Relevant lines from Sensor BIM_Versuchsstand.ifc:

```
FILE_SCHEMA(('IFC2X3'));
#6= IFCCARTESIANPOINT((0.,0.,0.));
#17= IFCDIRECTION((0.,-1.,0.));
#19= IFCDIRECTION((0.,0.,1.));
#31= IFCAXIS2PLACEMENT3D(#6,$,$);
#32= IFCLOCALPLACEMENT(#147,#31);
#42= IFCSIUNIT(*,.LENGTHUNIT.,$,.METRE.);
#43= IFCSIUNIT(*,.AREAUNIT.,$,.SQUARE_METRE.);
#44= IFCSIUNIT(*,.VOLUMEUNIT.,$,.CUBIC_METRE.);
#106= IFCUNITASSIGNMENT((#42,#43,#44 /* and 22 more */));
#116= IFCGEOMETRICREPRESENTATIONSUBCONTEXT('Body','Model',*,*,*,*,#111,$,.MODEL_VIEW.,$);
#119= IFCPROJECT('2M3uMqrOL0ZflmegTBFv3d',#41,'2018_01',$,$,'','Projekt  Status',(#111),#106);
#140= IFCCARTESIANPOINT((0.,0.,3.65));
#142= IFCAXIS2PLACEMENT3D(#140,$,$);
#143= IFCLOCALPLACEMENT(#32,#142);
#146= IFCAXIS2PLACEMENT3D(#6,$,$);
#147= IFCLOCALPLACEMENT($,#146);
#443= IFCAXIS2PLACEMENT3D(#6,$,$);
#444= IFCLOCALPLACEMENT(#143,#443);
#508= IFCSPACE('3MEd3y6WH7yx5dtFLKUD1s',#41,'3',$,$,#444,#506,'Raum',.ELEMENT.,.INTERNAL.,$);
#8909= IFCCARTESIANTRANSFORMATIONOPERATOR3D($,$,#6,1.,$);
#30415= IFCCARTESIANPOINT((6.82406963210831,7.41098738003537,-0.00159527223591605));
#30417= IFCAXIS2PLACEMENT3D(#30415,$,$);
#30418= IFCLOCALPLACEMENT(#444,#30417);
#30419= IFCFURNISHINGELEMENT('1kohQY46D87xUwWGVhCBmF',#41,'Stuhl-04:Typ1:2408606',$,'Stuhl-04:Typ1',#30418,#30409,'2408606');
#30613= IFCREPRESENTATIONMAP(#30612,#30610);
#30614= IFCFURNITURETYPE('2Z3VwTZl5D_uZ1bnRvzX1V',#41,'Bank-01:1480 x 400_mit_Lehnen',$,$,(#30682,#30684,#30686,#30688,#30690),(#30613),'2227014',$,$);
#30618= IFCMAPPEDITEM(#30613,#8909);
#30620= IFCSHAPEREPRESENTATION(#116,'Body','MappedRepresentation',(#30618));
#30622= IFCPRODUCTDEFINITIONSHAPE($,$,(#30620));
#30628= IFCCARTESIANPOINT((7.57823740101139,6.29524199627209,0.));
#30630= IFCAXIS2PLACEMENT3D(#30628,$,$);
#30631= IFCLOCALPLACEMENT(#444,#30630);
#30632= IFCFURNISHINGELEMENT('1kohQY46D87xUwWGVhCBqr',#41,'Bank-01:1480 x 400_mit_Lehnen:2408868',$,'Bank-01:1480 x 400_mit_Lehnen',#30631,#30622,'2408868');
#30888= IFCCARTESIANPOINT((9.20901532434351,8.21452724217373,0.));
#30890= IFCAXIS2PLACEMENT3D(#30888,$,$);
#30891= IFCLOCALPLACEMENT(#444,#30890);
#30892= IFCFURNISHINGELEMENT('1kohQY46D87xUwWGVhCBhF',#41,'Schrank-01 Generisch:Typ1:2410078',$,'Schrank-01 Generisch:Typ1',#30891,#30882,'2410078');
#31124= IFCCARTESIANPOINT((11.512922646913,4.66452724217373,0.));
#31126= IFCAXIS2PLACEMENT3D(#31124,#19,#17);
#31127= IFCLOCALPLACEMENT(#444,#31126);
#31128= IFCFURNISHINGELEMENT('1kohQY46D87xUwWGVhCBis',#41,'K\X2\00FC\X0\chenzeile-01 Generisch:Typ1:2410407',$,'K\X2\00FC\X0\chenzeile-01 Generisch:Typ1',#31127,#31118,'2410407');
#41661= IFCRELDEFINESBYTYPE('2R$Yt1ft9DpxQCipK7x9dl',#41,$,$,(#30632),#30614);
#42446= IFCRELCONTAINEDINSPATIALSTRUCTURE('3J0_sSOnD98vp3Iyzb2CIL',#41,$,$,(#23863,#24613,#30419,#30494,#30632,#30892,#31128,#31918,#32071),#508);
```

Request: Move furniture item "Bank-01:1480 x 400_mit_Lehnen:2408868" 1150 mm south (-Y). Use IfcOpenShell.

```python
import ifcopenshell
import ifcopenshell.api.geometry
import ifcopenshell.util.placement
import ifcopenshell.util.unit

model = ifcopenshell.open("Sensor BIM_Versuchsstand.ifc")
unit_scale = ifcopenshell.util.unit.calculate_unit_scale(model)

item = model.by_guid("1kohQY46D87xUwWGVhCBqr")
matrix = ifcopenshell.util.placement.get_local_placement(item.ObjectPlacement)
matrix[1, 3] -= 1.15 / unit_scale
ifcopenshell.api.geometry.edit_object_placement(model, product=item, matrix=matrix, is_si=False)

print(ifcopenshell.util.placement.get_local_placement(item.ObjectPlacement).round(3) + 0.0)

model.write("Sensor BIM_Versuchsstand_edited.ifc")
```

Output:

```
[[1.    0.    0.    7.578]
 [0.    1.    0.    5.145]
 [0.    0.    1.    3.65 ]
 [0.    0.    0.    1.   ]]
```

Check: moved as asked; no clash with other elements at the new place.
